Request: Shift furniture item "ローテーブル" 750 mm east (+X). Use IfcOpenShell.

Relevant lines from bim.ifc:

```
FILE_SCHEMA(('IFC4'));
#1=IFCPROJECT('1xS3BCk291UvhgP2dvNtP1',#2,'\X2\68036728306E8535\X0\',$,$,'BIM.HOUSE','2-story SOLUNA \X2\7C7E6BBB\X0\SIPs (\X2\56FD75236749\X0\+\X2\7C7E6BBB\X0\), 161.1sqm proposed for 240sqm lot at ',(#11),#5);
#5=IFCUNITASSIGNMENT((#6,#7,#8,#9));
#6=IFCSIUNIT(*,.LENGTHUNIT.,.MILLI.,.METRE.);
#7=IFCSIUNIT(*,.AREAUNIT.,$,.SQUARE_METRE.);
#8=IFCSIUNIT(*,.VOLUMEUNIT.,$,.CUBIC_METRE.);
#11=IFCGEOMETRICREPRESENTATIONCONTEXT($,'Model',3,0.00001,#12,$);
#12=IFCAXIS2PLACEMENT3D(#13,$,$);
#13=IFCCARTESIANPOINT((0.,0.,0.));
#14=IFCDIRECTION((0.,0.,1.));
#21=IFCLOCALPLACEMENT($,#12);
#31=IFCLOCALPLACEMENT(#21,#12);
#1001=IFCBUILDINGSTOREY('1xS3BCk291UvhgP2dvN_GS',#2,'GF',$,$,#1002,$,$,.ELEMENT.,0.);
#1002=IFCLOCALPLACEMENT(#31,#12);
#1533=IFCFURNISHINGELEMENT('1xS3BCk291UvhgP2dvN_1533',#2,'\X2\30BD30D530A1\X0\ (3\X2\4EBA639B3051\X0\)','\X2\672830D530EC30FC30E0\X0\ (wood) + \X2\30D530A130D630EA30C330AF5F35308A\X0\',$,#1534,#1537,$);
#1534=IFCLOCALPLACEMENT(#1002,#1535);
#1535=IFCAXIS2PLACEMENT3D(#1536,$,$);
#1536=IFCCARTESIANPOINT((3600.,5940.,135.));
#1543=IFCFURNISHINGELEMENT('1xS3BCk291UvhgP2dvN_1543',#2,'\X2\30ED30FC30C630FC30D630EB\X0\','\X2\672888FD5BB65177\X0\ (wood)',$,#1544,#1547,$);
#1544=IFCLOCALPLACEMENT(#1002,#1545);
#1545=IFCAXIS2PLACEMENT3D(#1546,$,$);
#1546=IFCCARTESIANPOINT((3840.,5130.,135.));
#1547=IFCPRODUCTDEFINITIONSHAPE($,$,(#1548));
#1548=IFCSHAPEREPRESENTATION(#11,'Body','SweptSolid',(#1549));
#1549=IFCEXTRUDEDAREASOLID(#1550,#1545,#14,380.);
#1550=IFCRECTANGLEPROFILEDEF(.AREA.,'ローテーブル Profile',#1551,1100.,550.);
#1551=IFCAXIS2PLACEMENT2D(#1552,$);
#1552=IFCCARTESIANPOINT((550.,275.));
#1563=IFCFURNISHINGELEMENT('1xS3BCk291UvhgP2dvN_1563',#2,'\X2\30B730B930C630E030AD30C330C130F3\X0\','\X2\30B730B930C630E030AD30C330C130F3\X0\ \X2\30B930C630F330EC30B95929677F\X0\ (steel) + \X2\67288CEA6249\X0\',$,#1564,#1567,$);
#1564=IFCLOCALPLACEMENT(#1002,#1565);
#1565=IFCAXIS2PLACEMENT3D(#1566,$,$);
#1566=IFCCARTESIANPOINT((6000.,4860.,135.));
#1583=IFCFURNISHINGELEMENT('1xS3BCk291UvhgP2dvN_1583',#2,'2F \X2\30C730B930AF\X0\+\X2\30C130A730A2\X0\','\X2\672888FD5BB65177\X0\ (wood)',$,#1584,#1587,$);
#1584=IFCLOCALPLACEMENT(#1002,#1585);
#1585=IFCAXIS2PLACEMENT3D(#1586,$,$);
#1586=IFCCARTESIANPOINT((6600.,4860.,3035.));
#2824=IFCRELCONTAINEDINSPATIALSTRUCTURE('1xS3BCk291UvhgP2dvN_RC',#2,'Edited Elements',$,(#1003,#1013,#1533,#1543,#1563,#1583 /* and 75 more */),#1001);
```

```python
import ifcopenshell
import ifcopenshell.api.geometry
import ifcopenshell.util.placement

model = ifcopenshell.open("bim.ifc")

item = model.by_id(1543)
matrix = ifcopenshell.util.placement.get_local_placement(item.ObjectPlacement)
matrix[0, 3] += 750.0
ifcopenshell.api.geometry.edit_object_placement(model, product=item, matrix=matrix, is_si=False)

print(ifcopenshell.util.placement.get_local_placement(item.ObjectPlacement).round(3) + 0.0)

model.write("bim-out.ifc")
```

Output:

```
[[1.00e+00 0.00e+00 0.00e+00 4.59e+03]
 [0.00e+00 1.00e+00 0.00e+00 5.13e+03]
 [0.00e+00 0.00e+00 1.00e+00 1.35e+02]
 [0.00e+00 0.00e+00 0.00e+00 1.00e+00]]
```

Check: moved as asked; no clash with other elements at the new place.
